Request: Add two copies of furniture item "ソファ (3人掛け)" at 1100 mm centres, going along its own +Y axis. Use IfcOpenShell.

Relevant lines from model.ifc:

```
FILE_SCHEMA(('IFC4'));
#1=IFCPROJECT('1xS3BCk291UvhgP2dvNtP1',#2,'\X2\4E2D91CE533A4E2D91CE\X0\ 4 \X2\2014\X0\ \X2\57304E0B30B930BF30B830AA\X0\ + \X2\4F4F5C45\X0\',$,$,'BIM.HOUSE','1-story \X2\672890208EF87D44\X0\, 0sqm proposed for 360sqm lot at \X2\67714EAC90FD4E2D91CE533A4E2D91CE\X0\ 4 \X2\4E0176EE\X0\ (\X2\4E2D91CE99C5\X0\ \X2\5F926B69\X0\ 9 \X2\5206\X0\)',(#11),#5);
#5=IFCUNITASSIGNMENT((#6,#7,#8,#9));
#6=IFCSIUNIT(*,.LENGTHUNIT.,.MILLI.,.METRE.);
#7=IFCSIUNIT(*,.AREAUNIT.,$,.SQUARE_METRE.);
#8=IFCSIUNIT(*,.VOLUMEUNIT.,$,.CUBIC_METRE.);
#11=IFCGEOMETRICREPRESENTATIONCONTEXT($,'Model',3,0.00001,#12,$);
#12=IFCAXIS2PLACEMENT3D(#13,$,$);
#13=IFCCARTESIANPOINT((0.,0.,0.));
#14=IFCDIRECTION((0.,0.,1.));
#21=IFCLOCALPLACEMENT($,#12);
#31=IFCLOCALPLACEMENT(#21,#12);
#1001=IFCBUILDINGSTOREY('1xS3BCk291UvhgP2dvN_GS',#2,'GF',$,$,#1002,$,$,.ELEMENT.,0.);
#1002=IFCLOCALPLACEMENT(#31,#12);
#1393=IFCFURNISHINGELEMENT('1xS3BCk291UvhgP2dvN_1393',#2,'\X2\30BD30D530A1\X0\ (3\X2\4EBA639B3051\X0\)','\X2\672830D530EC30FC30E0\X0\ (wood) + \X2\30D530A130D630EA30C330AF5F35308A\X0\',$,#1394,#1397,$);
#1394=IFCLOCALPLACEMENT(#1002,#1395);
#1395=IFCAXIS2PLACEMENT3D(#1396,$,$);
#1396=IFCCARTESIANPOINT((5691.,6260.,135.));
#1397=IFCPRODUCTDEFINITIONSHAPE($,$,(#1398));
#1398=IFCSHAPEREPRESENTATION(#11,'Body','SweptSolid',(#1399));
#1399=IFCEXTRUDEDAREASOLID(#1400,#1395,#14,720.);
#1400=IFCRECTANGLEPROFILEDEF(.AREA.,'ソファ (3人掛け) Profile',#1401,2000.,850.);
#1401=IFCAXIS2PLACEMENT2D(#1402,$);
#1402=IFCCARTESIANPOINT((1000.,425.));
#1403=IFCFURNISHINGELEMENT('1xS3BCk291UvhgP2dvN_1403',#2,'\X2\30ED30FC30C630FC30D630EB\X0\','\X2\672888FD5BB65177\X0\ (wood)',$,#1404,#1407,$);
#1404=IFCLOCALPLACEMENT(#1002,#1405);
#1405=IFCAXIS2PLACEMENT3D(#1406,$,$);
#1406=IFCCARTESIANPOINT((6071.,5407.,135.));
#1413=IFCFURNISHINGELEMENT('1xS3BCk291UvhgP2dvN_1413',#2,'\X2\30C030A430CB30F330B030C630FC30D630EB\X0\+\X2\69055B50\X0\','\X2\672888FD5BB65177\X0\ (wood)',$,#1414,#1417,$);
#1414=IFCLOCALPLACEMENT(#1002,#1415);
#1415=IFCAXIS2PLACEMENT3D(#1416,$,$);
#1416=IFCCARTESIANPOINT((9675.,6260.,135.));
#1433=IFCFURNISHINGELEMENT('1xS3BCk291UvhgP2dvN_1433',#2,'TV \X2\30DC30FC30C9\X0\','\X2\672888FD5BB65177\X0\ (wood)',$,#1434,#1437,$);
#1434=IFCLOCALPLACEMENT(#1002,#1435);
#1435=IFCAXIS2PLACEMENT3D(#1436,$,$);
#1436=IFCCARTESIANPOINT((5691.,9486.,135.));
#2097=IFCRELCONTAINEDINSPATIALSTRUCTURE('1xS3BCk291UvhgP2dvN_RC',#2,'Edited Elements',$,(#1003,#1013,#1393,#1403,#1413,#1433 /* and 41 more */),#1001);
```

```python
import ifcopenshell
import ifcopenshell.api.geometry
import ifcopenshell.api.root
import ifcopenshell.util.element
import ifcopenshell.util.placement
import ifcopenshell.util.unit

model = ifcopenshell.open("model.ifc")
unit_scale = ifcopenshell.util.unit.calculate_unit_scale(model)


def reuse_history(source, copy):
    """copy_class also copies each property set's owner history, people and application; keep the originals."""
    for rel in copy.IsDefinedBy:
        if rel.is_a("IfcRelDefinesByProperties") and (history := rel.RelatingPropertyDefinition.OwnerHistory):
            rel.RelatingPropertyDefinition.OwnerHistory = source.OwnerHistory
            ifcopenshell.util.element.remove_deep2(model, history)


source = model.by_guid("1xS3BCk291UvhgP2dvN_1393")
base = ifcopenshell.util.placement.get_local_placement(source.ObjectPlacement)
step = base[:3, 1] * 1.1 / unit_scale

for i in range(1, 3):
    copy = ifcopenshell.api.root.copy_class(model, product=source)
    copy.Representation = ifcopenshell.util.element.copy_deep(
        model, source.Representation, exclude=["IfcGeometricRepresentationContext", "IfcRepresentationMap"]
    )
    reuse_history(source, copy)
    matrix = base.copy()
    matrix[:3, 3] += i * step
    print("added at", matrix[:3, 3].round(3) + 0.0)
    ifcopenshell.api.geometry.edit_object_placement(model, product=copy, matrix=matrix, is_si=False)

model.write("model_v2.ifc")
```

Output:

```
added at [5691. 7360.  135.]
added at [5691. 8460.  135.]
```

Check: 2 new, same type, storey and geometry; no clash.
